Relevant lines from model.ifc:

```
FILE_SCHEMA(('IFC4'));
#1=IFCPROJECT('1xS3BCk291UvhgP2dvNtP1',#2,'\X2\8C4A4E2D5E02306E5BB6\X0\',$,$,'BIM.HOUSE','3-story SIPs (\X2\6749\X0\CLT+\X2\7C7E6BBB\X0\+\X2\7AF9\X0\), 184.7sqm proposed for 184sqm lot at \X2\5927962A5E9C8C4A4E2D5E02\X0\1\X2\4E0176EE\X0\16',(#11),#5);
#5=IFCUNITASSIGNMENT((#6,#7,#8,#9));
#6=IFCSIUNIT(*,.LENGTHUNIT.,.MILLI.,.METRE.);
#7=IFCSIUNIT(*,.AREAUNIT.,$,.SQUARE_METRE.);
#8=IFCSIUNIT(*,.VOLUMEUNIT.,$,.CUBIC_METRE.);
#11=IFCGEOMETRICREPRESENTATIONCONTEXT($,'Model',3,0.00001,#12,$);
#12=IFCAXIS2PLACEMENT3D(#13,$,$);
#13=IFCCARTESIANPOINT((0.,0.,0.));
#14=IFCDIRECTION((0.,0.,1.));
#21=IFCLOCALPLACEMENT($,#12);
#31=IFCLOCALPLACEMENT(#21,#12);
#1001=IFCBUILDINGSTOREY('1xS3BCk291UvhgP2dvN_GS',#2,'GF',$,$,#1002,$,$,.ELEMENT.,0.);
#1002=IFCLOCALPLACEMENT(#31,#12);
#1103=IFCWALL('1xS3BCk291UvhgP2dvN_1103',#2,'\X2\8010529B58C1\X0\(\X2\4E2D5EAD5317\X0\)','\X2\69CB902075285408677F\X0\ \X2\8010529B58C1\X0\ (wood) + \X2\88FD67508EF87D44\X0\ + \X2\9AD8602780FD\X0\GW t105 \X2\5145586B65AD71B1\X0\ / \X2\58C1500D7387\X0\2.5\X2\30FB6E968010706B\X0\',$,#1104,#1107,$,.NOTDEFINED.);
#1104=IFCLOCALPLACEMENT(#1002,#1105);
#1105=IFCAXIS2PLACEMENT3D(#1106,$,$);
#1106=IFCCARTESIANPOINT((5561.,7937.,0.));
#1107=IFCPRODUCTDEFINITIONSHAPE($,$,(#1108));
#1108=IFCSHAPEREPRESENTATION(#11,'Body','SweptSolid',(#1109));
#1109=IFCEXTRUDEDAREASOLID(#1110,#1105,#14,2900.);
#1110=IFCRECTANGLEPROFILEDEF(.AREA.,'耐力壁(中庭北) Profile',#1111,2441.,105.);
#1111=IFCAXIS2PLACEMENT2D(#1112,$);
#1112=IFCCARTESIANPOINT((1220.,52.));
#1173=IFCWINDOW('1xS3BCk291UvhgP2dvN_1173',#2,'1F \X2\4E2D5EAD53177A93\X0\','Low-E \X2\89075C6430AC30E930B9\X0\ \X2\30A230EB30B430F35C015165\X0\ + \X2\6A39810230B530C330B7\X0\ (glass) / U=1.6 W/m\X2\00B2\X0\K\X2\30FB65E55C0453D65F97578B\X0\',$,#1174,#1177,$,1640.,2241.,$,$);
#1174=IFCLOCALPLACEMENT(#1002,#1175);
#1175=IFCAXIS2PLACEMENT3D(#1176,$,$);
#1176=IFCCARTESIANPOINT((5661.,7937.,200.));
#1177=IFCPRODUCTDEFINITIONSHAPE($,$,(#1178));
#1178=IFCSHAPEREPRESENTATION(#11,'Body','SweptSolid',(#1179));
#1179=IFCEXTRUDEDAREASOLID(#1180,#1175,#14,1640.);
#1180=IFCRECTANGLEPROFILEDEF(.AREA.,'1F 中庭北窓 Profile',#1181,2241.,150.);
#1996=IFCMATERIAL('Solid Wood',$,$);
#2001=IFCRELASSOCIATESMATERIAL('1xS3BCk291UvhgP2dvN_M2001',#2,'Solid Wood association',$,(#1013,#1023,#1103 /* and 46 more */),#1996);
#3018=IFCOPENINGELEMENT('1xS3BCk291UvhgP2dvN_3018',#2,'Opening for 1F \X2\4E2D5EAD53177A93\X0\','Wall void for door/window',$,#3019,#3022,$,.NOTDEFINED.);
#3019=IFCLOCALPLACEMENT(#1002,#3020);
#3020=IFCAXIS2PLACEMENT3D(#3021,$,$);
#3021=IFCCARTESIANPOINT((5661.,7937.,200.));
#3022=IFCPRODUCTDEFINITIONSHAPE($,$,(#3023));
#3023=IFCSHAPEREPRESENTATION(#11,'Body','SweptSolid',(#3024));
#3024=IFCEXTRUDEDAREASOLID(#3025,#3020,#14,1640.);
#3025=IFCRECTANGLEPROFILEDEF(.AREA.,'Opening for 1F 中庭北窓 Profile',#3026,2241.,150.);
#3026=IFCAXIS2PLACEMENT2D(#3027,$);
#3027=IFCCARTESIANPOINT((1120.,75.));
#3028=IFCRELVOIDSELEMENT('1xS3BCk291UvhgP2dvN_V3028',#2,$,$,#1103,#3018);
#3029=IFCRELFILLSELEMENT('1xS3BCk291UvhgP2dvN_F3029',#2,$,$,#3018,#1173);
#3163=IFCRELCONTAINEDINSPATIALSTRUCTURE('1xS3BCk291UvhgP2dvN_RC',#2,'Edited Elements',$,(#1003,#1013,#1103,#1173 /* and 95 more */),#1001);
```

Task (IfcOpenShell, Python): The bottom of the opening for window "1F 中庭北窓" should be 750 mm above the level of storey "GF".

```python
import numpy as np
import ifcopenshell
import ifcopenshell.api.geometry
import ifcopenshell.geom
import ifcopenshell.util.element
import ifcopenshell.util.placement
import ifcopenshell.util.shape
import ifcopenshell.util.unit

model = ifcopenshell.open("model.ifc")
unit_scale = ifcopenshell.util.unit.calculate_unit_scale(model)

window = model.by_id(1173)
opening = window.FillsVoids[0].RelatingOpeningElement
storey = ifcopenshell.util.element.get_container(window, ifc_class="IfcBuildingStorey")
level = ifcopenshell.util.placement.get_local_placement(storey.ObjectPlacement)[2, 3]

# The opening's origin need not be at the sill, so measure its lowest point.
shape = ifcopenshell.geom.create_shape(ifcopenshell.geom.settings(), opening)
bottom = ifcopenshell.util.shape.get_shape_bottom_elevation(shape, shape.geometry) / unit_scale
dz = level + 0.75 / unit_scale - bottom

shift = np.array([0.0, 0.0, dz])
# The window is not placed relative to its opening, so move both.
for product in (opening, window):
    matrix = ifcopenshell.util.placement.get_local_placement(product.ObjectPlacement)
    matrix[:3, 3] += shift
    ifcopenshell.api.geometry.edit_object_placement(model, product=product, matrix=matrix, is_si=False)

print(f"moved by {dz * unit_scale:+.3f} m")

model.write("model_updated.ifc")
```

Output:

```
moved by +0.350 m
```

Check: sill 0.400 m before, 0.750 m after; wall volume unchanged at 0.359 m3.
